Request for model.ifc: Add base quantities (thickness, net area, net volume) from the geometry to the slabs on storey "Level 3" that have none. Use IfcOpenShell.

First a look at what the model holds.

```python
import ifcopenshell
import ifcopenshell.util.element
import ifcopenshell.util.unit

model = ifcopenshell.open("model.ifc")
print(model.schema)
for unit_type in ("LENGTHUNIT", "AREAUNIT", "VOLUMEUNIT"):
    print(unit_type, ifcopenshell.util.unit.calculate_unit_scale(model, unit_type))
storey = next(s for s in model.by_type("IfcBuildingStorey") if s.Name == "Level 3")
slabs = [e for e in ifcopenshell.util.element.get_decomposition(storey) if e.is_a("IfcSlab")]
for e in sorted(slabs, key=lambda e: e.id()):
    print(e.id(), e.is_a(), e.Name, list(ifcopenshell.util.element.get_psets(e, qtos_only=True)), sep=" | ")
```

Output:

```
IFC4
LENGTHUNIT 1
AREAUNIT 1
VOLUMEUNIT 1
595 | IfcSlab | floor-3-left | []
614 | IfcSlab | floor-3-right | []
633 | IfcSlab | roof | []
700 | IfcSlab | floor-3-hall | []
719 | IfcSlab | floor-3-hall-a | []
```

```python
import ifcopenshell
import ifcopenshell.api.pset
import ifcopenshell.geom
import ifcopenshell.util.element
import ifcopenshell.util.shape
import ifcopenshell.util.unit

model = ifcopenshell.open("model.ifc")
unit_scale = ifcopenshell.util.unit.calculate_unit_scale(model)
area_scale = ifcopenshell.util.unit.calculate_unit_scale(model, "AREAUNIT")
volume_scale = ifcopenshell.util.unit.calculate_unit_scale(model, "VOLUMEUNIT")
settings = ifcopenshell.geom.settings()

storey = next(s for s in model.by_type("IfcBuildingStorey") if s.Name == "Level 3")
slabs = [e for e in ifcopenshell.util.element.get_decomposition(storey) if e.is_a("IfcSlab")]

for e in sorted(slabs, key=lambda e: e.id()):
    if ifcopenshell.util.element.get_psets(e, qtos_only=True, should_inherit=False):
        continue
    # Geometry comes back in metres, in the element's own axes.
    shape = ifcopenshell.geom.create_shape(settings, e)
    values = {
        "Width": ifcopenshell.util.shape.get_z(shape.geometry) / unit_scale,
        "NetArea": ifcopenshell.util.shape.get_footprint_area(shape.geometry) / area_scale,
        "NetVolume": ifcopenshell.util.shape.get_volume(shape.geometry) / volume_scale,
    }
    qto = ifcopenshell.api.pset.add_qto(model, product=e, name="Qto_SlabBaseQuantities")
    ifcopenshell.api.pset.edit_qto(model, qto=qto, properties=values)
    print(e.id(), {k: round(v, 3) for k, v in values.items()})

model.write("model_updated.ifc")
```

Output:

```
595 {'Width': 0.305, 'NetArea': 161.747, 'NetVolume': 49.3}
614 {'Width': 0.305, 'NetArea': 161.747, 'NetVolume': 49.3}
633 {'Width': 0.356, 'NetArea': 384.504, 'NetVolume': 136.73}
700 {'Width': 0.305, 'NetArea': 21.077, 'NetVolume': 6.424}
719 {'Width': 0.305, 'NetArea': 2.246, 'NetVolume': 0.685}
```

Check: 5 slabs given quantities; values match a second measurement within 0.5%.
